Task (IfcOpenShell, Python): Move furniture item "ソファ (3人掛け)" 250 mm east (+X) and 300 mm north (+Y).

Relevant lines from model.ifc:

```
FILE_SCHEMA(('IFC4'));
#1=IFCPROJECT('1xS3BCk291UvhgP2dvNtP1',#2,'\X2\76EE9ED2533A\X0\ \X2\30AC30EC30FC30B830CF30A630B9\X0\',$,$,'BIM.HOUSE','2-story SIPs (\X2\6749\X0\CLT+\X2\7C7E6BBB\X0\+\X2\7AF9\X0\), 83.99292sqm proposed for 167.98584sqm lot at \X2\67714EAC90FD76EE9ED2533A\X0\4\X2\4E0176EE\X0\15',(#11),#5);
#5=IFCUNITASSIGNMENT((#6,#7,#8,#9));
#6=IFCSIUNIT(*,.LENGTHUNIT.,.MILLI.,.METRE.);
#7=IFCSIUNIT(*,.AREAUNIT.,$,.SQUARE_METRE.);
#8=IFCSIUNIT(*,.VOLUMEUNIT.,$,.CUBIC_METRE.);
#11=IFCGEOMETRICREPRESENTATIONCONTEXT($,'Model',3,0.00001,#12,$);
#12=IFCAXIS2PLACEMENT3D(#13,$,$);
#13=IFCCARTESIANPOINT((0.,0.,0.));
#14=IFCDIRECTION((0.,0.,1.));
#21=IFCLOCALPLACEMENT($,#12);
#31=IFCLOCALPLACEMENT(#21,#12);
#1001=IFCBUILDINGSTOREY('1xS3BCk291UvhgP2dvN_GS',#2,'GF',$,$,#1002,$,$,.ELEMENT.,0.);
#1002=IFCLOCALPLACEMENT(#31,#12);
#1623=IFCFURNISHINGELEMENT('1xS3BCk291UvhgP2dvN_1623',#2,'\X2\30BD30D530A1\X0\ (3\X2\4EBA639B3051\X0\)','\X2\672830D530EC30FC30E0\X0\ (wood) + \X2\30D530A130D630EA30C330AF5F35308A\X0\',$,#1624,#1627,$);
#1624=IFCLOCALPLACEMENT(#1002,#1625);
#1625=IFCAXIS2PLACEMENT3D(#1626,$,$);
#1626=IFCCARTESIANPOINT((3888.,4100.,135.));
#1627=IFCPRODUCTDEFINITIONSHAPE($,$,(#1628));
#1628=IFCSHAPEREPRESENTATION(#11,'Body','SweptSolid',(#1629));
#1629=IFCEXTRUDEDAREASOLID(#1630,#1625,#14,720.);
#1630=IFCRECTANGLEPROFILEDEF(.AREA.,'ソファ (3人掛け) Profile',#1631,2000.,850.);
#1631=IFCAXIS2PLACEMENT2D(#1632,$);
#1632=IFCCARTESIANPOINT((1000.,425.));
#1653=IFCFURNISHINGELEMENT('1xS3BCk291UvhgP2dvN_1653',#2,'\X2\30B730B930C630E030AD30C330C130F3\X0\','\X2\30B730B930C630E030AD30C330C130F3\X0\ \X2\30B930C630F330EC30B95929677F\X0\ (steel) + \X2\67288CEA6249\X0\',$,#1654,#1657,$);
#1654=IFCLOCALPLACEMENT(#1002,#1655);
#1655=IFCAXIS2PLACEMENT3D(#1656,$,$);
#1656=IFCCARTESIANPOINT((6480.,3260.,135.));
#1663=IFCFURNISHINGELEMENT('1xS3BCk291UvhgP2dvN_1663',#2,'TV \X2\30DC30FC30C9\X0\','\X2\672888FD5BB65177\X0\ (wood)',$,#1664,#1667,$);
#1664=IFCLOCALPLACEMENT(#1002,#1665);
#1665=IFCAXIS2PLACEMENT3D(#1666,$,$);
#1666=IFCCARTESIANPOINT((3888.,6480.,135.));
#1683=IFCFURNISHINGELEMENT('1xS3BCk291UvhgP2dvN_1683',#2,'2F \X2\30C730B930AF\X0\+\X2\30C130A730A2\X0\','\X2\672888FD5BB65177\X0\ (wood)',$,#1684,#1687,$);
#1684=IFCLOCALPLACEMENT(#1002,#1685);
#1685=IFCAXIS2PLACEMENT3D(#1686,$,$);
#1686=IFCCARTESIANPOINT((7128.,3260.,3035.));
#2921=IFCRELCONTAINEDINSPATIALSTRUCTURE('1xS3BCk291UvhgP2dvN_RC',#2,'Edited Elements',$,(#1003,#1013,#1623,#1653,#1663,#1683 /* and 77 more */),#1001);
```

```python
import ifcopenshell
import ifcopenshell.api.geometry
import ifcopenshell.util.placement

model = ifcopenshell.open("model.ifc")

item = model.by_guid("1xS3BCk291UvhgP2dvN_1623")
matrix = ifcopenshell.util.placement.get_local_placement(item.ObjectPlacement)
matrix[0, 3] += 250.0
matrix[1, 3] += 300.0
ifcopenshell.api.geometry.edit_object_placement(model, product=item, matrix=matrix, is_si=False)

print(ifcopenshell.util.placement.get_local_placement(item.ObjectPlacement).round(3) + 0.0)

model.write("model_rev.ifc")
```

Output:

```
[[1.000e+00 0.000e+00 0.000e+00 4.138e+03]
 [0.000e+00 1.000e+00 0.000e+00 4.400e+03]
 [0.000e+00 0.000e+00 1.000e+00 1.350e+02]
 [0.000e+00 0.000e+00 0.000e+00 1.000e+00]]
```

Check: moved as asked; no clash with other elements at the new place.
